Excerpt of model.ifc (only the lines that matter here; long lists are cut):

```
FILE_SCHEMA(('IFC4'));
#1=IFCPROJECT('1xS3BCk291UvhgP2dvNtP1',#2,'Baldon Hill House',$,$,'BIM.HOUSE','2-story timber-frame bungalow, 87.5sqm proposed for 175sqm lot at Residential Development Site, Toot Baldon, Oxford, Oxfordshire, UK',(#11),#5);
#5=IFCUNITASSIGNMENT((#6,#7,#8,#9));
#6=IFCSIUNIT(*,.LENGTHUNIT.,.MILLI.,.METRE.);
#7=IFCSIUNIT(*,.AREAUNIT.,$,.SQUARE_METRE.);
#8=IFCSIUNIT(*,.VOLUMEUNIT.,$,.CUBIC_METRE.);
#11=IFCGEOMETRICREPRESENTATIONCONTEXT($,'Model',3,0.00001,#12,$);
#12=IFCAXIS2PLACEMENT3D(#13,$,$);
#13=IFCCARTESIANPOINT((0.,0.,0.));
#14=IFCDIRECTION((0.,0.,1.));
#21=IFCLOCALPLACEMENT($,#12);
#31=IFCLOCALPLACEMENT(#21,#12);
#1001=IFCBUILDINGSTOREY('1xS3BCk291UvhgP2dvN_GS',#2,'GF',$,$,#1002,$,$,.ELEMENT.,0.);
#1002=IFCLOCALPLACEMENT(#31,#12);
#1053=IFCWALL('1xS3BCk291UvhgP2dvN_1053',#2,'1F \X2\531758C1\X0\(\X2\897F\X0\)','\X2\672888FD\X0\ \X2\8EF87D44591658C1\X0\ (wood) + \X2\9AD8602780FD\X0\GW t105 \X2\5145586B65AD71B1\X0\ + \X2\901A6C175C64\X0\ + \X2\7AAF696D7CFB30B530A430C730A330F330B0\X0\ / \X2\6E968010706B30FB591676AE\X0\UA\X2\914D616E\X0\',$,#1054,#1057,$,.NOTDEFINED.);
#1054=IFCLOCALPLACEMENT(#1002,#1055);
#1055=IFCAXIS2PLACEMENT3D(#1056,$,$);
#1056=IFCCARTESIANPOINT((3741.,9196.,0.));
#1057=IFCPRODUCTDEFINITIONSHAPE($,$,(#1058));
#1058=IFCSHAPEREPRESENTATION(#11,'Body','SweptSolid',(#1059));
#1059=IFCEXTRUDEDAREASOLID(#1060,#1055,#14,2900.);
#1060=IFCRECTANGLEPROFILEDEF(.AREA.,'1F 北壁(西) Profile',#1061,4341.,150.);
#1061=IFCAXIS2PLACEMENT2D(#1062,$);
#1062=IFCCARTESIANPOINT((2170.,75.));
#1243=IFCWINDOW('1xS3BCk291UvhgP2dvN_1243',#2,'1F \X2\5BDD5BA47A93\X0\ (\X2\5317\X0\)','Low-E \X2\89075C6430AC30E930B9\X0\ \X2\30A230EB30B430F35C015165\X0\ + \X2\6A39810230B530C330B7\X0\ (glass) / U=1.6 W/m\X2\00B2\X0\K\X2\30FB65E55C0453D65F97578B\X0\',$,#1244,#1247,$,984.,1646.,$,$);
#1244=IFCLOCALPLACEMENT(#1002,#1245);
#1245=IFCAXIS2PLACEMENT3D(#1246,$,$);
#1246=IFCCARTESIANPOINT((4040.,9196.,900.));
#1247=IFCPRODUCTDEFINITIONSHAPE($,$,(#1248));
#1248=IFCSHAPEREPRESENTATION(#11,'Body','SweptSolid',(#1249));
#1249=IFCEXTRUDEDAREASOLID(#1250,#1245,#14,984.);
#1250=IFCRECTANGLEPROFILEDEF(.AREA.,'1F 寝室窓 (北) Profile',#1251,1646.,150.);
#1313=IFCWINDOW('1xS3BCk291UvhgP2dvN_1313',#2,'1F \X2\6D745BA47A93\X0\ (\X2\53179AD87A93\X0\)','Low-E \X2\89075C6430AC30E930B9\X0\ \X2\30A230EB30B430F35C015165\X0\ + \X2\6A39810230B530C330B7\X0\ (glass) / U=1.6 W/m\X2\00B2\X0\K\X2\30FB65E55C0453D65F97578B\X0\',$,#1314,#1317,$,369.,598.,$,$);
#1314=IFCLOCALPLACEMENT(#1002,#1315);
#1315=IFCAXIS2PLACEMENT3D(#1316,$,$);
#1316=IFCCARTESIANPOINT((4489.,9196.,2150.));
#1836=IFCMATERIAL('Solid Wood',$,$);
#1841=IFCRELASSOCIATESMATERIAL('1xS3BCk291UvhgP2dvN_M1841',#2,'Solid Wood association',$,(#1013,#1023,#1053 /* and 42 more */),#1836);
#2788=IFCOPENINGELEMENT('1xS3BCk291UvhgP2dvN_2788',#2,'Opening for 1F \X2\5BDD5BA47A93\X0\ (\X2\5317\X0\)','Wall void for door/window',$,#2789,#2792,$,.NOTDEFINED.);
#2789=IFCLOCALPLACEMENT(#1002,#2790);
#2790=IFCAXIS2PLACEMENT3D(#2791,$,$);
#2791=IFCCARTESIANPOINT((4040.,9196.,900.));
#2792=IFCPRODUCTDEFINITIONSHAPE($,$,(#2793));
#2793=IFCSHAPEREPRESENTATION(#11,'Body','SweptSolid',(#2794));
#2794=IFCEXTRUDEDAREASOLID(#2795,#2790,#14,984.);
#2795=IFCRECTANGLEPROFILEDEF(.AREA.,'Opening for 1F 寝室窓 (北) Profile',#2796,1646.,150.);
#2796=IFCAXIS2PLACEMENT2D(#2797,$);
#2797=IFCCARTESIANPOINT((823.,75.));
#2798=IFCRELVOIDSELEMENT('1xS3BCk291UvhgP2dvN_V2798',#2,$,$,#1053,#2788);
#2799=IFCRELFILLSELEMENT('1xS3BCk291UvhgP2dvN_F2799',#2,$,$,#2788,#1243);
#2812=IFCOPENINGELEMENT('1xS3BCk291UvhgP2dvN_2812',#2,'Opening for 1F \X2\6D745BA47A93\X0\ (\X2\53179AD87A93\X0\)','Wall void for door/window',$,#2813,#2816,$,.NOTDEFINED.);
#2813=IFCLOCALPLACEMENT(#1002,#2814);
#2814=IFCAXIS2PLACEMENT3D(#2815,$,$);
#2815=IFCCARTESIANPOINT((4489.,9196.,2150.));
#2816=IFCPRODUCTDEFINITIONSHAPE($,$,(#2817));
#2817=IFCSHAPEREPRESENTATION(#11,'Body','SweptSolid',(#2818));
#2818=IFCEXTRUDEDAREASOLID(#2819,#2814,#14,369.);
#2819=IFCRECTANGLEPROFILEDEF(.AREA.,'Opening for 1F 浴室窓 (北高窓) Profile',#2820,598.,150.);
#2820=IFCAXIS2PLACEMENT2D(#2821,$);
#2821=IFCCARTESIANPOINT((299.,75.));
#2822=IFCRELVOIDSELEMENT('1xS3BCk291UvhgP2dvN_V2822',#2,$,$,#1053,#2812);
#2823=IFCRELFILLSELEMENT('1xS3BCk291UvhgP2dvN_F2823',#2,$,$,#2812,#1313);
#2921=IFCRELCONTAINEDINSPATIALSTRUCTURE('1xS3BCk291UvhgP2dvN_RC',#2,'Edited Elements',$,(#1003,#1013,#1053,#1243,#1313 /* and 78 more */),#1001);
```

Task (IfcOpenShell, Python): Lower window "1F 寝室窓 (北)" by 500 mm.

```python
import numpy as np
import ifcopenshell
import ifcopenshell.api.geometry
import ifcopenshell.util.placement
import ifcopenshell.util.unit

model = ifcopenshell.open("model.ifc")
unit_scale = ifcopenshell.util.unit.calculate_unit_scale(model)

window = model.by_guid("1xS3BCk291UvhgP2dvN_1243")
opening = window.FillsVoids[0].RelatingOpeningElement
dz = -500.0

shift = np.array([0.0, 0.0, dz])
# The window is not placed relative to its opening, so move both.
for product in (opening, window):
    matrix = ifcopenshell.util.placement.get_local_placement(product.ObjectPlacement)
    matrix[:3, 3] += shift
    ifcopenshell.api.geometry.edit_object_placement(model, product=product, matrix=matrix, is_si=False)

print(f"moved by {dz * unit_scale:+.3f} m")

model.write("model_v2.ifc")
```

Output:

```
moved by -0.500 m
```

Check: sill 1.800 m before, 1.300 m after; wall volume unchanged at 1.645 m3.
